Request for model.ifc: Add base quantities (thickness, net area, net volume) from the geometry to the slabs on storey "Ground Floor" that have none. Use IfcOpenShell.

First a look at what the model holds.

```python
import ifcopenshell
import ifcopenshell.util.element
import ifcopenshell.util.unit

model = ifcopenshell.open("model.ifc")
print(model.schema)
for unit_type in ("LENGTHUNIT", "AREAUNIT", "VOLUMEUNIT"):
    print(unit_type, ifcopenshell.util.unit.calculate_unit_scale(model, unit_type))
storey = next(s for s in model.by_type("IfcBuildingStorey") if s.Name == "Ground Floor")
slabs = [e for e in ifcopenshell.util.element.get_decomposition(storey) if e.is_a("IfcSlab")]
for e in sorted(slabs, key=lambda e: e.id()):
    print(e.id(), e.is_a(), e.Name, list(ifcopenshell.util.element.get_psets(e, qtos_only=True)), sep=" | ")
```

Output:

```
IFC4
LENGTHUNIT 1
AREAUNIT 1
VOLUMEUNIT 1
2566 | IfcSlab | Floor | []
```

```python
import ifcopenshell
import ifcopenshell.api.pset
import ifcopenshell.geom
import ifcopenshell.util.element
import ifcopenshell.util.shape
import ifcopenshell.util.unit

model = ifcopenshell.open("model.ifc")
unit_scale = ifcopenshell.util.unit.calculate_unit_scale(model)
area_scale = ifcopenshell.util.unit.calculate_unit_scale(model, "AREAUNIT")
volume_scale = ifcopenshell.util.unit.calculate_unit_scale(model, "VOLUMEUNIT")
settings = ifcopenshell.geom.settings()

storey = next(s for s in model.by_type("IfcBuildingStorey") if s.Name == "Ground Floor")
slabs = [e for e in ifcopenshell.util.element.get_decomposition(storey) if e.is_a("IfcSlab")]

for e in sorted(slabs, key=lambda e: e.id()):
    if ifcopenshell.util.element.get_psets(e, qtos_only=True, should_inherit=False):
        continue
    # Geometry comes back in metres, in the element's own axes.
    shape = ifcopenshell.geom.create_shape(settings, e)
    values = {
        "Width": ifcopenshell.util.shape.get_z(shape.geometry) / unit_scale,
        "NetArea": ifcopenshell.util.shape.get_footprint_area(shape.geometry) / area_scale,
        "NetVolume": ifcopenshell.util.shape.get_volume(shape.geometry) / volume_scale,
    }
    qto = ifcopenshell.api.pset.add_qto(model, product=e, name="Qto_SlabBaseQuantities")
    ifcopenshell.api.pset.edit_qto(model, qto=qto, properties=values)
    print(e.id(), {k: round(v, 3) for k, v in values.items()})

model.write("model_rev.ifc")
```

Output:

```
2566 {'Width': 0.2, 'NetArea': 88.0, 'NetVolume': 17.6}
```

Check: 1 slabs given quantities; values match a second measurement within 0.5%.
